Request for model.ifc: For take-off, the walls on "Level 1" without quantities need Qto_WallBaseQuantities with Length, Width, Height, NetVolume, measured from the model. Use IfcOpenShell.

First a look at what the model holds.

```python
import ifcopenshell
import ifcopenshell.util.element
import ifcopenshell.util.unit

model = ifcopenshell.open("model.ifc")
print(model.schema)
for unit_type in ("LENGTHUNIT", "AREAUNIT", "VOLUMEUNIT"):
    print(unit_type, ifcopenshell.util.unit.calculate_unit_scale(model, unit_type))
storey = next(s for s in model.by_type("IfcBuildingStorey") if s.Name == "Level 1")
walls = [e for e in ifcopenshell.util.element.get_decomposition(storey) if e.is_a("IfcWall")]
for e in sorted(walls, key=lambda e: e.id()):
    print(e.id(), e.is_a(), e.Name, list(ifcopenshell.util.element.get_psets(e, qtos_only=True)), sep=" | ")
```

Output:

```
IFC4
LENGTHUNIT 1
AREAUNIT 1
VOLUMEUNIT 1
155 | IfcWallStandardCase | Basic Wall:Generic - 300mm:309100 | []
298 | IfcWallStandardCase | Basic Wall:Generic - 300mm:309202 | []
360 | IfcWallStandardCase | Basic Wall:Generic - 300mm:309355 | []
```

```python
import ifcopenshell
import ifcopenshell.api.pset
import ifcopenshell.geom
import ifcopenshell.util.element
import ifcopenshell.util.shape
import ifcopenshell.util.unit

model = ifcopenshell.open("model.ifc")
unit_scale = ifcopenshell.util.unit.calculate_unit_scale(model)
volume_scale = ifcopenshell.util.unit.calculate_unit_scale(model, "VOLUMEUNIT")
settings = ifcopenshell.geom.settings()

storey = next(s for s in model.by_type("IfcBuildingStorey") if s.Name == "Level 1")
walls = [e for e in ifcopenshell.util.element.get_decomposition(storey) if e.is_a("IfcWall")]

for e in sorted(walls, key=lambda e: e.id()):
    if ifcopenshell.util.element.get_psets(e, qtos_only=True, should_inherit=False):
        continue
    # Geometry comes back in metres, in the element's own axes.
    shape = ifcopenshell.geom.create_shape(settings, e)
    values = {
        "Length": ifcopenshell.util.shape.get_x(shape.geometry) / unit_scale,
        "Width": ifcopenshell.util.shape.get_y(shape.geometry) / unit_scale,
        "Height": ifcopenshell.util.shape.get_z(shape.geometry) / unit_scale,
        "NetVolume": ifcopenshell.util.shape.get_volume(shape.geometry) / volume_scale,
    }
    qto = ifcopenshell.api.pset.add_qto(model, product=e, name="Qto_WallBaseQuantities")
    ifcopenshell.api.pset.edit_qto(model, qto=qto, properties=values)
    print(e.id(), {k: round(v, 3) for k, v in values.items()})

model.write("model_updated.ifc")
```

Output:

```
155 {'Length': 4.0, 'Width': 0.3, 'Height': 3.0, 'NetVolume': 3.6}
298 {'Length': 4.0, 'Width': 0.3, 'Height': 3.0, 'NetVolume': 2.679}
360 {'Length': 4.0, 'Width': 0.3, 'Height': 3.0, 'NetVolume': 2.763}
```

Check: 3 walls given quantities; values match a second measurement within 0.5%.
